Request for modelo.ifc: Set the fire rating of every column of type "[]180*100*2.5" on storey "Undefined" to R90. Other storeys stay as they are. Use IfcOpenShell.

First a look at what the model holds.

```python
import ifcopenshell
import ifcopenshell.util.element

model = ifcopenshell.open("modelo.ifc")
print(model.schema)
storey = next(s for s in model.by_type("IfcBuildingStorey") if s.Name == "Undefined")
columns = [e for e in ifcopenshell.util.element.get_decomposition(storey) if e.is_a("IfcColumn")]
seen = {}
for e in columns:
    element_type = ifcopenshell.util.element.get_type(e)
    key = (element_type.Name if element_type != e and element_type else None, ifcopenshell.util.element.get_pset(e, "Pset_ColumnCommon", "FireRating"))
    seen[key] = seen.get(key, 0) + 1
for (name, value), count in sorted(seen.items(), key=str):
    print(count, "x", name, "|", value)
```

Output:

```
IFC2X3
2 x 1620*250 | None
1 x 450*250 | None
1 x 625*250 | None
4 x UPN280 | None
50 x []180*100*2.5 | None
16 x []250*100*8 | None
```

```python
import ifcopenshell
import ifcopenshell.api.pset
import ifcopenshell.util.element

model = ifcopenshell.open("modelo.ifc")

storey = next(s for s in model.by_type("IfcBuildingStorey") if s.Name == "Undefined")
columns = [e for e in ifcopenshell.util.element.get_decomposition(storey) if e.is_a("IfcColumn")]

count = 0
for e in columns:
    element_type = ifcopenshell.util.element.get_type(e)
    if element_type in (None, e) or element_type.Name != "[]180*100*2.5":
        continue
    found = ifcopenshell.util.element.get_pset(e, "Pset_ColumnCommon", should_inherit=False)
    if found:
        pset = model.by_id(found["id"])
        if len(ifcopenshell.util.element.get_elements_by_pset(pset)) > 1:
            pset = ifcopenshell.api.pset.unshare_pset(model, products=[e], pset=pset)[0]
    else:
        pset = ifcopenshell.api.pset.add_pset(model, product=e, name="Pset_ColumnCommon")
    ifcopenshell.api.pset.edit_pset(model, pset=pset, properties={"FireRating": "R90"})
    count += 1

print(count, "columns updated")

model.write("modelo_rev.ifc")
```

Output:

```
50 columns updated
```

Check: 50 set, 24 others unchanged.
